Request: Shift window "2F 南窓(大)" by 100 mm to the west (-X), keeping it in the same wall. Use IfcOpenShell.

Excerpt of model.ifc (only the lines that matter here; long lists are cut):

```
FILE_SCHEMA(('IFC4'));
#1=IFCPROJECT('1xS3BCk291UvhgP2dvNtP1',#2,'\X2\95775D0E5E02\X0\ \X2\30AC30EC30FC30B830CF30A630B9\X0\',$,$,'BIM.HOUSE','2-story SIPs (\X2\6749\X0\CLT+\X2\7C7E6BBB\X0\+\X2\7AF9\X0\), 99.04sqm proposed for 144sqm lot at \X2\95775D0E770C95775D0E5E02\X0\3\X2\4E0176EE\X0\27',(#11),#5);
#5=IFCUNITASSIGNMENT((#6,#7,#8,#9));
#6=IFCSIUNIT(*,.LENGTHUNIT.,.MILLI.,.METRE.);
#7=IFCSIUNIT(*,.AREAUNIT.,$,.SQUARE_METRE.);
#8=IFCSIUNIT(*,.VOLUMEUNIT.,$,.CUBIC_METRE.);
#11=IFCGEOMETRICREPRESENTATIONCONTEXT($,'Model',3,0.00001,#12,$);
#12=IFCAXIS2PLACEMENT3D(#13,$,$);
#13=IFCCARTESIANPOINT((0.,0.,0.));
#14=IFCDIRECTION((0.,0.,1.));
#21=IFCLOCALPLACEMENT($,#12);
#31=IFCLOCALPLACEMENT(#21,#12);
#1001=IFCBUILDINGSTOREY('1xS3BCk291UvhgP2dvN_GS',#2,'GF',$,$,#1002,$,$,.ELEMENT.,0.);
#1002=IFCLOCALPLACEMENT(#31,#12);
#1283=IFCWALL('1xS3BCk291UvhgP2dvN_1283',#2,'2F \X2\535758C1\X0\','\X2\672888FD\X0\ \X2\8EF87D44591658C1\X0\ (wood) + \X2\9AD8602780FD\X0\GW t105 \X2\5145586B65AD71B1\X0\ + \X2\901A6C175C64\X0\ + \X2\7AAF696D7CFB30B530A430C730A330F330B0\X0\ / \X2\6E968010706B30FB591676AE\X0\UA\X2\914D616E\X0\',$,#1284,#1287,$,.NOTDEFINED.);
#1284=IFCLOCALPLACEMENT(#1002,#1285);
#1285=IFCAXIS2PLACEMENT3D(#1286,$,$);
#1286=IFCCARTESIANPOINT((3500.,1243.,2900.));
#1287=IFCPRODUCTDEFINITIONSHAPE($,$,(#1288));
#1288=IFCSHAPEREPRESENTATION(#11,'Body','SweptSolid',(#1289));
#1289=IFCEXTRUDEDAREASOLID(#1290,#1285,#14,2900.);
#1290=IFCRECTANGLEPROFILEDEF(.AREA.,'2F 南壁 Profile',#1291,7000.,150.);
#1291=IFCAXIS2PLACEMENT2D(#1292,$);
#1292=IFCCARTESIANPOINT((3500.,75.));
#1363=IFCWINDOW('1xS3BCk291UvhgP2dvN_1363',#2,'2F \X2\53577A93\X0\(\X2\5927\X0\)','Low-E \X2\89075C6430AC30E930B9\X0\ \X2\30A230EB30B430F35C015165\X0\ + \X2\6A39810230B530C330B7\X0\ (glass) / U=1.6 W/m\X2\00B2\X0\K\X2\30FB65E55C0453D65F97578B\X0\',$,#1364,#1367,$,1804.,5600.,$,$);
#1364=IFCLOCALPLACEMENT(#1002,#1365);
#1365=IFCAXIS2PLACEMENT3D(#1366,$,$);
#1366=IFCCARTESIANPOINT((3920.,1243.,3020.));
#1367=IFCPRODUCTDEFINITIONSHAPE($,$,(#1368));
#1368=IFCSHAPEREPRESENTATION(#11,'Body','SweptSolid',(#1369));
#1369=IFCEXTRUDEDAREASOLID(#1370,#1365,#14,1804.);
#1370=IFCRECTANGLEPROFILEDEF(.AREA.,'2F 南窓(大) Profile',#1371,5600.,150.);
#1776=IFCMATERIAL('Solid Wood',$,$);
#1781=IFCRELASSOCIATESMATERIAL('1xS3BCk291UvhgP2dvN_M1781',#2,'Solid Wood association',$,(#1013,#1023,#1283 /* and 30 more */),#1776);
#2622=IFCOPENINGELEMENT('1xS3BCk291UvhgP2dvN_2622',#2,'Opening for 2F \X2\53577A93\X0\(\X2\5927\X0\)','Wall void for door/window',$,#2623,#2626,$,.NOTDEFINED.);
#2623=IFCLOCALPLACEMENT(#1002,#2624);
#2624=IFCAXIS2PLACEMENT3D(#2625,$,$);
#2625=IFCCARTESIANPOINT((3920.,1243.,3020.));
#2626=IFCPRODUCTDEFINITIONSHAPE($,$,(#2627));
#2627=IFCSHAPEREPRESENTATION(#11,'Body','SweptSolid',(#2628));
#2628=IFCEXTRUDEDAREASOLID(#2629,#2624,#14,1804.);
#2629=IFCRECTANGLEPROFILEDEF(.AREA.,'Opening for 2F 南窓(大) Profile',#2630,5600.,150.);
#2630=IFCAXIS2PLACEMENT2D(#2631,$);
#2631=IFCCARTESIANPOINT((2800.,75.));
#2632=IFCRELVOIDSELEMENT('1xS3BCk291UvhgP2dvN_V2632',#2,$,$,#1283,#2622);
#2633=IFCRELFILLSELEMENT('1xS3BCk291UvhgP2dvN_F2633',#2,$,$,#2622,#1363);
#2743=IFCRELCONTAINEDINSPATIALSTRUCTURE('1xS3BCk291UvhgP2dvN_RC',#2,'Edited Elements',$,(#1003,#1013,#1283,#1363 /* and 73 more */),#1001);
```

```python
import ifcopenshell
import ifcopenshell.api.geometry
import ifcopenshell.util.placement
import ifcopenshell.util.unit

model = ifcopenshell.open("model.ifc")
unit_scale = ifcopenshell.util.unit.calculate_unit_scale(model)

window = model.by_guid("1xS3BCk291UvhgP2dvN_1363")
opening = window.FillsVoids[0].RelatingOpeningElement
wall = opening.VoidsElements[0].RelatingBuildingElement

wall_matrix = ifcopenshell.util.placement.get_local_placement(wall.ObjectPlacement)
shift = wall_matrix[:3, 0] * -0.1 / unit_scale
before = ifcopenshell.util.placement.get_local_placement(window.ObjectPlacement)[:3, 3].copy()

# The window is not placed relative to its opening, so move both.
for product in (opening, window):
    matrix = ifcopenshell.util.placement.get_local_placement(product.ObjectPlacement)
    matrix[:3, 3] += shift
    ifcopenshell.api.geometry.edit_object_placement(model, product=product, matrix=matrix, is_si=False)

after = ifcopenshell.util.placement.get_local_placement(window.ObjectPlacement)[:3, 3]
print("window moved by", (after - before).round(3) + 0.0)

model.write("model-out.ifc")
```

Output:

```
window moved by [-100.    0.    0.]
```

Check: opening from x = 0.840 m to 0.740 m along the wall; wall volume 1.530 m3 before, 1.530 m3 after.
